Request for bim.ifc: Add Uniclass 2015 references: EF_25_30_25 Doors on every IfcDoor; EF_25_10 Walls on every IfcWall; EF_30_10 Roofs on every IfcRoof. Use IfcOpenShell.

First a look at what the model holds.

```python
import ifcopenshell

model = ifcopenshell.open("bim.ifc")
print(model.schema)
print("classifications:", [c.Name for c in model.by_type("IfcClassification")])
for ifc_class in ("IfcDoor", "IfcRoof", "IfcStair", "IfcWall", "IfcWindow"):
    print(ifc_class, len(model.by_type(ifc_class)))
```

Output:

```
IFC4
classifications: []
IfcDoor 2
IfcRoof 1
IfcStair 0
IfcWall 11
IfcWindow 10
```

```python
import ifcopenshell
import ifcopenshell.api.classification

model = ifcopenshell.open("bim.ifc")

system = ifcopenshell.api.classification.add_classification(model, classification="Uniclass 2015")

codes = {
    "IfcDoor": ("EF_25_30_25", "Doors"),
    "IfcWall": ("EF_25_10", "Walls"),
    "IfcRoof": ("EF_30_10", "Roofs"),
}
for ifc_class, (code, name) in codes.items():
    products = model.by_type(ifc_class)
    ifcopenshell.api.classification.add_reference(
        model, products=products, classification=system, identification=code, name=name
    )
    print(code, len(products))

model.write("bim_rev.ifc")
```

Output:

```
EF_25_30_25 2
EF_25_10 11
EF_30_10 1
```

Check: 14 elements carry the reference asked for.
